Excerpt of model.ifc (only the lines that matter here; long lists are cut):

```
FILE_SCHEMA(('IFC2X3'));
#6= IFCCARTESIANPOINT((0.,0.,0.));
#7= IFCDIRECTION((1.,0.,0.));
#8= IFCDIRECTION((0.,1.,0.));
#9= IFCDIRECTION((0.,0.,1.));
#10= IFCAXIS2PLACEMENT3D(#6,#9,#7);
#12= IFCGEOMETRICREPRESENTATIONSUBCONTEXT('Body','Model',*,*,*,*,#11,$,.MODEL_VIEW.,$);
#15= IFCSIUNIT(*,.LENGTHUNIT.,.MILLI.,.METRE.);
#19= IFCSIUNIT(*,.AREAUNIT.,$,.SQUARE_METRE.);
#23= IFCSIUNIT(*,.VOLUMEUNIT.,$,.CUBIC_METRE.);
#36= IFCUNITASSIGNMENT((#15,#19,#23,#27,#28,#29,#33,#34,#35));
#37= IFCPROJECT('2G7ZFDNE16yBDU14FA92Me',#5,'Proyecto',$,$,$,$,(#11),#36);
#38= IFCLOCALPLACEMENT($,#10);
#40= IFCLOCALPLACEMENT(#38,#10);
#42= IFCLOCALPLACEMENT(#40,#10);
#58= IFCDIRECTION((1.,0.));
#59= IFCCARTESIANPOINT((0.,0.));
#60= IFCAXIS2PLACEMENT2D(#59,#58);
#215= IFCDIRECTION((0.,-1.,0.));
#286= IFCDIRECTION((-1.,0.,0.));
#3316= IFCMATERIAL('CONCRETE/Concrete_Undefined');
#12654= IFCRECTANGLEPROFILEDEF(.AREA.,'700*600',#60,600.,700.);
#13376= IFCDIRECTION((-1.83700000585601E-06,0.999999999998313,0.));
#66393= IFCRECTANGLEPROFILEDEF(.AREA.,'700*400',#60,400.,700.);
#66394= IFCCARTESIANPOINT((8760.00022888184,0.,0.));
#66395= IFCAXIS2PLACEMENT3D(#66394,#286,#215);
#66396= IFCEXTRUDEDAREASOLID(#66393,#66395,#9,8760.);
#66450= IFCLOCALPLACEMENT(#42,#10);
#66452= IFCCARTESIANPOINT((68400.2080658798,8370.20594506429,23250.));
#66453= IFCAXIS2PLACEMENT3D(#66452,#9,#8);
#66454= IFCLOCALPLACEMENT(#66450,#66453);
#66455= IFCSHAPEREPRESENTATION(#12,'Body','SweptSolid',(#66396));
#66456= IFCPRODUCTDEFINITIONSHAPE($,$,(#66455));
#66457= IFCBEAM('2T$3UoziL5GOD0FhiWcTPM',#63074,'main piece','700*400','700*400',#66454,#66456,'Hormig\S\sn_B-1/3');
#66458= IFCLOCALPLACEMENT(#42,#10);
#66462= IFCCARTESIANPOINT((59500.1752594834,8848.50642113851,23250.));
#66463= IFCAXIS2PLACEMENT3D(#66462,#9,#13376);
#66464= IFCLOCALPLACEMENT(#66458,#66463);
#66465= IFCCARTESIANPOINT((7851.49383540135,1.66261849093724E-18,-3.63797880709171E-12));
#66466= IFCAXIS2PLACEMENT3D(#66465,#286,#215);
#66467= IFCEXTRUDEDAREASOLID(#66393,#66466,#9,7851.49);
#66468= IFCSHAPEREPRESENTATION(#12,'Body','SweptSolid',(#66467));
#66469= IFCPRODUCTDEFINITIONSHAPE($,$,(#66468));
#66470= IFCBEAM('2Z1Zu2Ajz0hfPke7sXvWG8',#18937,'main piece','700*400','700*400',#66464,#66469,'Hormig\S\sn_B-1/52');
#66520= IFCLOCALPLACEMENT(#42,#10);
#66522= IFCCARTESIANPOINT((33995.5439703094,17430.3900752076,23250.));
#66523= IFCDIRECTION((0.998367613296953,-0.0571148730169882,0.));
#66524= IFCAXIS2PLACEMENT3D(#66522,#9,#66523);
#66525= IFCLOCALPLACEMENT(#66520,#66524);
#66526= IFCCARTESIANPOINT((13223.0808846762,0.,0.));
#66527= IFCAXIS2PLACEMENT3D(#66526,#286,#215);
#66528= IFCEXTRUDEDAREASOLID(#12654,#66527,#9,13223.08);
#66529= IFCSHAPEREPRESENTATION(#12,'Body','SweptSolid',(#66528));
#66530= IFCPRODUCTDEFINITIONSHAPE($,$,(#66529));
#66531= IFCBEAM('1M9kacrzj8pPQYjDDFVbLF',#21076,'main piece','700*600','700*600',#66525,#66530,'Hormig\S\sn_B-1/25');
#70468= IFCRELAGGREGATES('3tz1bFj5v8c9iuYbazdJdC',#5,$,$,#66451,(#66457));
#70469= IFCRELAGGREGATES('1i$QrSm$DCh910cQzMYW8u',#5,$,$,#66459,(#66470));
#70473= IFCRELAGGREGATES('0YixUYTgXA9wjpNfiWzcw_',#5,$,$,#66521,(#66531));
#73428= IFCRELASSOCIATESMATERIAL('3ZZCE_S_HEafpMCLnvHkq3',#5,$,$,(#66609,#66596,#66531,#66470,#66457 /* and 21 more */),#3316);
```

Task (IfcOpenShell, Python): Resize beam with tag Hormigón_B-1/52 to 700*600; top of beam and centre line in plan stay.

```python
import ifcopenshell
import ifcopenshell.util.element
import ifcopenshell.util.representation

model = ifcopenshell.open("model.ifc")

member = model.by_id(66470)
source = next(p for p in model.by_type("IfcRectangleProfileDef") if p.ProfileName == "700*600")

body = ifcopenshell.util.representation.get_representation(member, "Model", "Body")
solid = body.Items[0]
old_profile = solid.SweptArea

# Copy the section's sizes but keep this member's own profile position.
profile = ifcopenshell.util.element.copy(model, source)
# Profiles are centred, so shift by half the change in depth to hold the top.
shift = (old_profile.YDim - profile.YDim) / 2
x, y = old_profile.Position.Location.Coordinates
up = (0.0, 1.0)  # upwards, in the solid's own plane
location = model.createIfcCartesianPoint((x + up[0] * shift, y + up[1] * shift))
profile.Position = model.createIfcAxis2Placement2D(location, old_profile.Position.RefDirection)
solid.SweptArea = profile
if not model.get_total_inverses(old_profile):
    ifcopenshell.util.element.remove_deep2(model, old_profile)
member.Description = member.Description.replace("700*400", "700*600")
member.ObjectType = member.ObjectType.replace("700*400", "700*600")

print(solid.SweptArea)

model.write("model_updated.ifc")
```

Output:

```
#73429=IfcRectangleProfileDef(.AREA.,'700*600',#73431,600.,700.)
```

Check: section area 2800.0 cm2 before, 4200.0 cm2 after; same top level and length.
